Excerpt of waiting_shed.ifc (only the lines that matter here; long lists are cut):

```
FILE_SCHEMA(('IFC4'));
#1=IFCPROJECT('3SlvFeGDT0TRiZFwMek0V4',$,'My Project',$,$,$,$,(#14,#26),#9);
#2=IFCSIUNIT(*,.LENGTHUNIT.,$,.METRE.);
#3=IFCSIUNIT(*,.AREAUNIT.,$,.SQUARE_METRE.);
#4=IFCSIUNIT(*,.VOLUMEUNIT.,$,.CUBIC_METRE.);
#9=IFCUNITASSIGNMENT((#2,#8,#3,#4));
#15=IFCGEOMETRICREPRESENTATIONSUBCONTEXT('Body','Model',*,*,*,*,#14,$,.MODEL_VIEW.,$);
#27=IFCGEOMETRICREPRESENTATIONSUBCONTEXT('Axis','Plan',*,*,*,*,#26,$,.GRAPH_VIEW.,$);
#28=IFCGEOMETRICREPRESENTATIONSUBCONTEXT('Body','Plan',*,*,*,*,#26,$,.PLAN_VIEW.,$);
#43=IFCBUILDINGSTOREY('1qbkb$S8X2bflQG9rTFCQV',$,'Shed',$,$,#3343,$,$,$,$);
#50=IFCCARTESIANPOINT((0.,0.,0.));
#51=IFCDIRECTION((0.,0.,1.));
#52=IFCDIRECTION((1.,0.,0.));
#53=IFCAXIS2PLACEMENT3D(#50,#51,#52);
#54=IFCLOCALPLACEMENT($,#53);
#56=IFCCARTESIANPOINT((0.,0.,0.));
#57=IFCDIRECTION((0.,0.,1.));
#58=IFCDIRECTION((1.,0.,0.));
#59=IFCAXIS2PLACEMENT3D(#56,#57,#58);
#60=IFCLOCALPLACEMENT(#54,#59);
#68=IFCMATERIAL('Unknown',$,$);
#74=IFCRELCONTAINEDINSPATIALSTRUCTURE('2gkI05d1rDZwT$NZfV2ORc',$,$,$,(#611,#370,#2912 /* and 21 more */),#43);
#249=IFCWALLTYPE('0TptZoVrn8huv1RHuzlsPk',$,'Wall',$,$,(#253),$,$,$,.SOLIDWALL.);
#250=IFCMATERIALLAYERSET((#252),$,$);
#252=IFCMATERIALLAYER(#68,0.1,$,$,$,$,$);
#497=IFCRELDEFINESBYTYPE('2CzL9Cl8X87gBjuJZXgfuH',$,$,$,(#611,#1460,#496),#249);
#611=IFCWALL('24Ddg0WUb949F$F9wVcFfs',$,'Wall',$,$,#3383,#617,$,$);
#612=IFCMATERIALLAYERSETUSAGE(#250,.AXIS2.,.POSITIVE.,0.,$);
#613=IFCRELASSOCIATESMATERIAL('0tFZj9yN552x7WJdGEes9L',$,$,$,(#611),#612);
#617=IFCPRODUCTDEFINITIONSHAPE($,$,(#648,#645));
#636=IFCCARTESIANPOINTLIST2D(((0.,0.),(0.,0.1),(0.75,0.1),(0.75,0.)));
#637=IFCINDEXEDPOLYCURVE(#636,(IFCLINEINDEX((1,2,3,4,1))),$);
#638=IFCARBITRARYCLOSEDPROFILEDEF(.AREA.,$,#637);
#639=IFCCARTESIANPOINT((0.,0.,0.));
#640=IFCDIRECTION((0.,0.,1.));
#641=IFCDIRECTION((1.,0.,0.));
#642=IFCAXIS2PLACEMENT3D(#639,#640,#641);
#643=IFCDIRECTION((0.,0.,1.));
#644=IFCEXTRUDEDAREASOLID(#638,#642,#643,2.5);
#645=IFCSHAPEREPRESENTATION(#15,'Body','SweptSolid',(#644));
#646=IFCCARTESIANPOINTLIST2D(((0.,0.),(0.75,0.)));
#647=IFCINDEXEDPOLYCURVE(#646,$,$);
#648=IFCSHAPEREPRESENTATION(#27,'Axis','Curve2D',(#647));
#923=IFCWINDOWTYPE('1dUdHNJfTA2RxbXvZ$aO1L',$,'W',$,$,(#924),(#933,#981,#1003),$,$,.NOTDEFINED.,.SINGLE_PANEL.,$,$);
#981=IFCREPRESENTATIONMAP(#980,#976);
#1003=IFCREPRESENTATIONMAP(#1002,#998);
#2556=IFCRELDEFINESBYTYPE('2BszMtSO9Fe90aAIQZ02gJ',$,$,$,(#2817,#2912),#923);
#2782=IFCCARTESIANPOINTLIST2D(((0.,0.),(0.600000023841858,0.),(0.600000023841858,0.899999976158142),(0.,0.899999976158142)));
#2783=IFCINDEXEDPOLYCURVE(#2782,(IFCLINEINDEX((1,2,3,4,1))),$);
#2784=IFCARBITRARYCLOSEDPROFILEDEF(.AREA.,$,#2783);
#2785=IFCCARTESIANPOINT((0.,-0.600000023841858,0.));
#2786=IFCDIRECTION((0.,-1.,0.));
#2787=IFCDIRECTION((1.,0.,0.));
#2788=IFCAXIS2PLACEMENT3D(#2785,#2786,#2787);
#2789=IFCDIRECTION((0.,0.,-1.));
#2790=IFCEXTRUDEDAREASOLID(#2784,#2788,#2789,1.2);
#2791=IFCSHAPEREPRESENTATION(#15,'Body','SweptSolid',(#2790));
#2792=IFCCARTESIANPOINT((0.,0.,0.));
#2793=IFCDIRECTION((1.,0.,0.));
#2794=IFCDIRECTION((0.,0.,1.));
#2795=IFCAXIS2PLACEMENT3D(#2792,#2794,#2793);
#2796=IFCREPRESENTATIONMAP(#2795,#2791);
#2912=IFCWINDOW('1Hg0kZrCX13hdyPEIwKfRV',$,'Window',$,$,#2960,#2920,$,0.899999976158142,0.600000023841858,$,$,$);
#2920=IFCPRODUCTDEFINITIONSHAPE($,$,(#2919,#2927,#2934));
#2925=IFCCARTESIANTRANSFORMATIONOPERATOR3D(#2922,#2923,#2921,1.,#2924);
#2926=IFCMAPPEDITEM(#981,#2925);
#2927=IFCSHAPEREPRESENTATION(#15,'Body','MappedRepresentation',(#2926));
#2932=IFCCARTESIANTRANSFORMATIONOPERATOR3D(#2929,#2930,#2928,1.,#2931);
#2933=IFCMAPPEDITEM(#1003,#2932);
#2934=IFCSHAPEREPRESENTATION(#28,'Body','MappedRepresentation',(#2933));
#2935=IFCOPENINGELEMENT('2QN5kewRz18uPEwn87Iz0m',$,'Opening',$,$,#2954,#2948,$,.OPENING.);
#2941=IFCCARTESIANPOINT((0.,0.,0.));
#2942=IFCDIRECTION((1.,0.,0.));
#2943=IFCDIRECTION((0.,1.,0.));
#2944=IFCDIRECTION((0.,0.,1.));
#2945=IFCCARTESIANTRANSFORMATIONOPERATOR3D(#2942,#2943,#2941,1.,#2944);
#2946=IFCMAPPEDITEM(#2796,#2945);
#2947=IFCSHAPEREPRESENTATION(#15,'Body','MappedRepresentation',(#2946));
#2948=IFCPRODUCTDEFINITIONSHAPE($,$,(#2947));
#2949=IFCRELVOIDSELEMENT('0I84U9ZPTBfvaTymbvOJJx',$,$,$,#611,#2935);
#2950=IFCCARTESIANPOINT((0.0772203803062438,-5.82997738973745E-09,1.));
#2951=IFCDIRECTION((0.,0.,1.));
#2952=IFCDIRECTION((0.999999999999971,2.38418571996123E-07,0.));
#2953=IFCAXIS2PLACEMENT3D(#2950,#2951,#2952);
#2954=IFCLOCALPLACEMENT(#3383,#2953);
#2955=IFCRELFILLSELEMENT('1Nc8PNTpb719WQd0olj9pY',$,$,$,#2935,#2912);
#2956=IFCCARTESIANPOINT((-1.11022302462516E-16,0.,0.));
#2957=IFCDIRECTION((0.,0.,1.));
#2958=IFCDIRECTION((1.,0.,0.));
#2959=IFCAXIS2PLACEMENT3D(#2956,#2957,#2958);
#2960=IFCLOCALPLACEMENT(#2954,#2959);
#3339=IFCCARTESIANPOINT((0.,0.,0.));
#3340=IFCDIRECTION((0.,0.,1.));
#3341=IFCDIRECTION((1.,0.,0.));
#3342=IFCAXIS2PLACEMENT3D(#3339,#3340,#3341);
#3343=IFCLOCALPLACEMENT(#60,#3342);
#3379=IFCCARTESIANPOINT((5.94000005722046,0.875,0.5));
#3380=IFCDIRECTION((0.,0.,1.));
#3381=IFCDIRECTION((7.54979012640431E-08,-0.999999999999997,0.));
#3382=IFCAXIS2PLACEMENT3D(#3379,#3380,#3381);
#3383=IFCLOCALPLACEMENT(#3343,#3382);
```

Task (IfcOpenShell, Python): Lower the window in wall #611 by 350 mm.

```python
import numpy as np
import ifcopenshell
import ifcopenshell.api.geometry
import ifcopenshell.util.placement
import ifcopenshell.util.unit

model = ifcopenshell.open("waiting_shed.ifc")
unit_scale = ifcopenshell.util.unit.calculate_unit_scale(model)

window = model.by_guid("1Hg0kZrCX13hdyPEIwKfRV")
opening = window.FillsVoids[0].RelatingOpeningElement
dz = -0.35 / unit_scale

shift = np.array([0.0, 0.0, dz])
# The window is placed relative to its opening, so it follows when the opening moves.
matrix = ifcopenshell.util.placement.get_local_placement(opening.ObjectPlacement)
matrix[:3, 3] += shift
ifcopenshell.api.geometry.edit_object_placement(
    model, product=opening, matrix=matrix, is_si=False, should_transform_children=True
)

print(f"moved by {dz * unit_scale:+.3f} m")

model.write("waiting_shed_v2.ifc")
```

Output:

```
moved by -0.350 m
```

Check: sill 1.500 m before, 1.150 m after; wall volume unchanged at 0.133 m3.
